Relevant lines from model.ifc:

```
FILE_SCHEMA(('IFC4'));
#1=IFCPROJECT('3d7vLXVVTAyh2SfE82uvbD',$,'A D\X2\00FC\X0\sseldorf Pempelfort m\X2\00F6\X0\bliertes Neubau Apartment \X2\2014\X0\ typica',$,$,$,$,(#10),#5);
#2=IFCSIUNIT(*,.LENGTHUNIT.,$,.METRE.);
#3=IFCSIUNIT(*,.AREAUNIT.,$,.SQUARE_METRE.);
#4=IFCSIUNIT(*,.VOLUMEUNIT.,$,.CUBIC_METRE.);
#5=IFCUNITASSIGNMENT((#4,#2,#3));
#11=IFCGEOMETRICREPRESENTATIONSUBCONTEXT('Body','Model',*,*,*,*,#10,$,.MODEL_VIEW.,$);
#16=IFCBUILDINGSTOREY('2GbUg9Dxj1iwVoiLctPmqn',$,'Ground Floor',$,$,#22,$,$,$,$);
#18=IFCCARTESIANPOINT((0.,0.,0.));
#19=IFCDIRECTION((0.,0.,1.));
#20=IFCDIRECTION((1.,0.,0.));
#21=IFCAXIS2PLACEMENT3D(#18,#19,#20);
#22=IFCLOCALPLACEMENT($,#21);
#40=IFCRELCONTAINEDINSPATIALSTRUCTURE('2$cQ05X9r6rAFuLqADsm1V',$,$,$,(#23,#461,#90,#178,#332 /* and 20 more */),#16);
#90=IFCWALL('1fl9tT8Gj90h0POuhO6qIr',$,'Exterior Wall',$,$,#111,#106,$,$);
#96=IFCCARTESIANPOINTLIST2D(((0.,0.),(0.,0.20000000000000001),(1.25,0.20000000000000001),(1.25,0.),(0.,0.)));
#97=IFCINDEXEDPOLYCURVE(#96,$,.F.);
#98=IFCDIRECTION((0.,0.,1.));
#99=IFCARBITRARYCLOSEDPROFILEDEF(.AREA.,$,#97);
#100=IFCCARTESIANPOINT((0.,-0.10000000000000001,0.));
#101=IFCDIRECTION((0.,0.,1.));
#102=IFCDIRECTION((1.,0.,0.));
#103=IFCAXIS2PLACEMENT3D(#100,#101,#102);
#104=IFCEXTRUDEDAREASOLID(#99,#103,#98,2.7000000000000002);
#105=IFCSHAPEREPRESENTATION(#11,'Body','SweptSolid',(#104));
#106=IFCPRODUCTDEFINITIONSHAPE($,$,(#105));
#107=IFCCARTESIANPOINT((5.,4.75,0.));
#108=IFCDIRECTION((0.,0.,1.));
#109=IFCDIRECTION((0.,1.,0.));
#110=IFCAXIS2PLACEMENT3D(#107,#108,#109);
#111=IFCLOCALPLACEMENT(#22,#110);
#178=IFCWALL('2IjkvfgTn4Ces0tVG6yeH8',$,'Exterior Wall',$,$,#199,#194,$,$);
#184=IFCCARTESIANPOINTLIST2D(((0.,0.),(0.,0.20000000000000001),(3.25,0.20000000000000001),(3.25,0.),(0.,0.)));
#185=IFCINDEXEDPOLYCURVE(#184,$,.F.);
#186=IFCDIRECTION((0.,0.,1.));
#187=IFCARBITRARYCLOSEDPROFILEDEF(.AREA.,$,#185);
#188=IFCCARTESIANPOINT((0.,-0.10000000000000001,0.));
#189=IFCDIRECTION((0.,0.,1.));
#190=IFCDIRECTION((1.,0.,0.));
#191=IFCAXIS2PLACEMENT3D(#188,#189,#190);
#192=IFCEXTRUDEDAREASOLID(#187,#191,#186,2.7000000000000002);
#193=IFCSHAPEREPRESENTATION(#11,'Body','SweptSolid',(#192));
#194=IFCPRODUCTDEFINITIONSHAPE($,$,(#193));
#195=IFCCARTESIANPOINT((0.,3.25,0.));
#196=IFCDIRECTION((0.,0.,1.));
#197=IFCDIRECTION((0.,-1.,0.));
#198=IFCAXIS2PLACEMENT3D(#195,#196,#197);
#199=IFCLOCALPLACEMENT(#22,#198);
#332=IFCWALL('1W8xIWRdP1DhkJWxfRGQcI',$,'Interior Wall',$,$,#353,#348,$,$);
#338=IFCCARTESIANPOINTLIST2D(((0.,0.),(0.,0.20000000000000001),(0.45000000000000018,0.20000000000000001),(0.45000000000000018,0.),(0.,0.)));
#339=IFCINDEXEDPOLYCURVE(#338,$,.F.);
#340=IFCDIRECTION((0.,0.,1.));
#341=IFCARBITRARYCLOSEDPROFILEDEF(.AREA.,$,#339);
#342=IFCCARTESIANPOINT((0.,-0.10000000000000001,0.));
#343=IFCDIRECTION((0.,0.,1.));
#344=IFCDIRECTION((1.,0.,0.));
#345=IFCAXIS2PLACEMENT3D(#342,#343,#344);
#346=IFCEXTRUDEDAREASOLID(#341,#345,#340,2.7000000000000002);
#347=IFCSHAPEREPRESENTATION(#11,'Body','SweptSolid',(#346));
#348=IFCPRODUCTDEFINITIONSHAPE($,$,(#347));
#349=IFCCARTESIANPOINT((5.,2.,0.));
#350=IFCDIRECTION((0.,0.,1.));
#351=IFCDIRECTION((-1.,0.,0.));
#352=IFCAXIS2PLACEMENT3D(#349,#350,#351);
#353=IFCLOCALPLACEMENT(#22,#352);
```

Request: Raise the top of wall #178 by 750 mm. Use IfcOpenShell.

```python
import ifcopenshell
import ifcopenshell.geom
import ifcopenshell.util.representation
import ifcopenshell.util.shape
import ifcopenshell.util.unit

model = ifcopenshell.open("model.ifc")
unit_scale = ifcopenshell.util.unit.calculate_unit_scale(model)
settings = ifcopenshell.geom.settings()


def volume(element):
    """Net volume in cubic metres, openings subtracted."""
    shape = ifcopenshell.geom.create_shape(settings, element)
    return ifcopenshell.util.shape.get_volume(shape.geometry)


wall = model.by_guid("2IjkvfgTn4Ces0tVG6yeH8")
before = volume(wall)

body = ifcopenshell.util.representation.get_representation(wall, "Model", "Body")
solid = body.Items[0]
old_height = solid.Depth
solid.Depth += 0.75 / unit_scale
after = volume(wall)

print(f"height {old_height:g} -> {solid.Depth:g}, volume {before:.3f} -> {after:.3f} m3")

model.write("model_v2.ifc")
```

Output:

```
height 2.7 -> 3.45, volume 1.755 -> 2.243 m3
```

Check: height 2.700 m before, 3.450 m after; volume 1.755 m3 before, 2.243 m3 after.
